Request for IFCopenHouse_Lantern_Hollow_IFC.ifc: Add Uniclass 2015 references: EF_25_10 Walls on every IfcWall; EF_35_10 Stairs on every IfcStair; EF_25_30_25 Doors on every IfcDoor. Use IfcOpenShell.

First a look at what the model holds.

```python
import ifcopenshell

model = ifcopenshell.open("IFCopenHouse_Lantern_Hollow_IFC.ifc")
print(model.schema)
print("classifications:", [c.Name for c in model.by_type("IfcClassification")])
for ifc_class in ("IfcDoor", "IfcRoof", "IfcStair", "IfcWall", "IfcWindow"):
    print(ifc_class, len(model.by_type(ifc_class)))
```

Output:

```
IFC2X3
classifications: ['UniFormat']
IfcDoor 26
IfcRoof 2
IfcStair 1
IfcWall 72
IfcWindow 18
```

```python
import ifcopenshell
import ifcopenshell.api.classification

model = ifcopenshell.open("IFCopenHouse_Lantern_Hollow_IFC.ifc")

# IFC2X3 requires Source and Edition and has no link from the project to the system.
system = model.create_entity("IfcClassification", Source="NBS", Edition="2015", Name="Uniclass 2015")

codes = {
    "IfcWall": ("EF_25_10", "Walls"),
    "IfcStair": ("EF_35_10", "Stairs"),
    "IfcDoor": ("EF_25_30_25", "Doors"),
}
for ifc_class, (code, name) in codes.items():
    products = model.by_type(ifc_class)
    ifcopenshell.api.classification.add_reference(
        model, products=products, classification=system, identification=code, name=name
    )
    print(code, len(products))

model.write("IFCopenHouse_Lantern_Hollow_IFC_v2.ifc")
```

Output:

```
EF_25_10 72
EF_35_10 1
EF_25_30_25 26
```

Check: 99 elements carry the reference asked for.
